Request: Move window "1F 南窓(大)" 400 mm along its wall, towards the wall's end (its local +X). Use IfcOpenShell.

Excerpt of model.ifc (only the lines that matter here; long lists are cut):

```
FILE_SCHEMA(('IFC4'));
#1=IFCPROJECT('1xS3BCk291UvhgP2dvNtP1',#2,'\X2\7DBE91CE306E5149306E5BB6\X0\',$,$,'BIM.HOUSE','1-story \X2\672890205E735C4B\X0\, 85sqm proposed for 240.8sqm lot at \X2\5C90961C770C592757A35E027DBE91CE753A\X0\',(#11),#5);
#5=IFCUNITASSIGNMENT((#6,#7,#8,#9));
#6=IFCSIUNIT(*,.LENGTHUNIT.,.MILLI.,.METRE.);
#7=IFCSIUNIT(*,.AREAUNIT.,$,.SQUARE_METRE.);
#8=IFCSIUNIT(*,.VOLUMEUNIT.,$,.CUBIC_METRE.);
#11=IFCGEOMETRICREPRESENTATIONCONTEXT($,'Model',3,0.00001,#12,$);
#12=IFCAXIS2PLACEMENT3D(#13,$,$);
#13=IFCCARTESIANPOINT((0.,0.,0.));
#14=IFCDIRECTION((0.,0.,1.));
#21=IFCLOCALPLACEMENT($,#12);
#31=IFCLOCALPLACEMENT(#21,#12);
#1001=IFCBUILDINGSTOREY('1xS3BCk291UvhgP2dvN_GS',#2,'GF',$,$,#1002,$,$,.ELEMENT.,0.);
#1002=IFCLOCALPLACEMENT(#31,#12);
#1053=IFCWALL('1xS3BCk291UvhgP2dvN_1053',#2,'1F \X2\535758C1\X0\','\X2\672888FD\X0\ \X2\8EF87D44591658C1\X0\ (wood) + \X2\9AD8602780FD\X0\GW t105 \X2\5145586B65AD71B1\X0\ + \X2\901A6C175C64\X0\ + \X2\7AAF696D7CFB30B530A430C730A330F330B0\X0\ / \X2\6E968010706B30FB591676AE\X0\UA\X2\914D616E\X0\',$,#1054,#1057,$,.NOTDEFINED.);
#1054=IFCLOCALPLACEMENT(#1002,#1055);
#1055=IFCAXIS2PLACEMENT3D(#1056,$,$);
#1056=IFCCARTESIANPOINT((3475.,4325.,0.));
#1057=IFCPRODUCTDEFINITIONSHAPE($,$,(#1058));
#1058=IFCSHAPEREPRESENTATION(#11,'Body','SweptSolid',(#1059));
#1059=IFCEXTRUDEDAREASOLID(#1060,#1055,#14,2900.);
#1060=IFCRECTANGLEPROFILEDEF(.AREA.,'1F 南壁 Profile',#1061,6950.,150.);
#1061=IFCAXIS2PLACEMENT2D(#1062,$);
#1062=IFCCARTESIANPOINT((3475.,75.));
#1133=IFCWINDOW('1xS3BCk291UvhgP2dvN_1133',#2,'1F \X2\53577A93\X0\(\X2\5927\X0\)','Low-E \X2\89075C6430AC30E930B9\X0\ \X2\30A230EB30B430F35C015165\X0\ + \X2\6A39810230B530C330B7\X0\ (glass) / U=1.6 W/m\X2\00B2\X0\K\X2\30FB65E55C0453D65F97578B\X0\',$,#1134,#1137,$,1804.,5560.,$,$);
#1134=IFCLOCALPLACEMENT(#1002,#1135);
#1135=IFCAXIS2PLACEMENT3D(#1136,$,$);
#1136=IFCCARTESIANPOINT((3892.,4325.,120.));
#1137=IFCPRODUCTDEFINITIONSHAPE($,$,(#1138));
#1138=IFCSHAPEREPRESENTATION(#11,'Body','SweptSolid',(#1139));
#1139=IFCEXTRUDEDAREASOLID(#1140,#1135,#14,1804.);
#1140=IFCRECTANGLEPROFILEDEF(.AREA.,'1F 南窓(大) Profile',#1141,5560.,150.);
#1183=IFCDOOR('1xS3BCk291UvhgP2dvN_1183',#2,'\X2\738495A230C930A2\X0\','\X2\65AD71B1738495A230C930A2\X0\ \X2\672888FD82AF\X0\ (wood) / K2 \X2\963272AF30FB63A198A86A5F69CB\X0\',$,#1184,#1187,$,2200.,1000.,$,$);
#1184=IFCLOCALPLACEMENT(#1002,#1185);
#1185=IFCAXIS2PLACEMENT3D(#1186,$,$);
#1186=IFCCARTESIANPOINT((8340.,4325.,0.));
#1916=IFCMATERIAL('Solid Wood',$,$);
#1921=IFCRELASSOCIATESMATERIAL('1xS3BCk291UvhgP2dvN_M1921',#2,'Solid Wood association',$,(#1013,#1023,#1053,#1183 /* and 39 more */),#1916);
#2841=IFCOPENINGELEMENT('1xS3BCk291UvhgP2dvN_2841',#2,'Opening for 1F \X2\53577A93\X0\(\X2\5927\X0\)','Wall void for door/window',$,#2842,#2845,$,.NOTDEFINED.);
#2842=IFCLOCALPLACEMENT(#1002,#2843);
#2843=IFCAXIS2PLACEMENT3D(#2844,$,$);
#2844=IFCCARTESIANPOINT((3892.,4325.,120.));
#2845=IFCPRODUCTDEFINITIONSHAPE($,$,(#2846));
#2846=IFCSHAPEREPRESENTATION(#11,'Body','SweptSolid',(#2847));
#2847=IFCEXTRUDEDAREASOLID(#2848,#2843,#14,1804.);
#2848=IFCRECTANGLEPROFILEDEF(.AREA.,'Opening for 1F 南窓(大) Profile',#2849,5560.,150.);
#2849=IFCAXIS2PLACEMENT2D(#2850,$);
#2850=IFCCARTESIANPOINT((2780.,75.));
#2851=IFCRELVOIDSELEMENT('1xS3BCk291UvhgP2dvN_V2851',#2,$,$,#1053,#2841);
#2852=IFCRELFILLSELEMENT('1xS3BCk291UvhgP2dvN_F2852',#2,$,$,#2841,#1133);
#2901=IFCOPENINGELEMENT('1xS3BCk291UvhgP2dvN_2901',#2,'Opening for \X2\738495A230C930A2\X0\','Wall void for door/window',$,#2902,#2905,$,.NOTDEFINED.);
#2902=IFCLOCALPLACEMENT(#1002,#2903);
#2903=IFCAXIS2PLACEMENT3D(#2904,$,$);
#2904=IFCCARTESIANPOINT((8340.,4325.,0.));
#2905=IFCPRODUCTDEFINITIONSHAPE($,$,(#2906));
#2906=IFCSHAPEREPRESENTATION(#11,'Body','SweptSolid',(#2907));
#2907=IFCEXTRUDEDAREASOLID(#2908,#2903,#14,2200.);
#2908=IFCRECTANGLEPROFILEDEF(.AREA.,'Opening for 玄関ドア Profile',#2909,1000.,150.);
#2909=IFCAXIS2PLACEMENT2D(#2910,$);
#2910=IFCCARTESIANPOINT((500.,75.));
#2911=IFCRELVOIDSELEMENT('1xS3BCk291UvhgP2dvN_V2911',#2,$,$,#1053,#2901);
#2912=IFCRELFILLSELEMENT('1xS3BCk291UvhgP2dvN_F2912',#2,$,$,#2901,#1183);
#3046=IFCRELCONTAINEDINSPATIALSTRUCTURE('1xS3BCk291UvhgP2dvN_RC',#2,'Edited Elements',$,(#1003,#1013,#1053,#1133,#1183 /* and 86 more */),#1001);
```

```python
import ifcopenshell
import ifcopenshell.api.geometry
import ifcopenshell.util.placement

model = ifcopenshell.open("model.ifc")

window = model.by_guid("1xS3BCk291UvhgP2dvN_1133")
opening = window.FillsVoids[0].RelatingOpeningElement
wall = opening.VoidsElements[0].RelatingBuildingElement

wall_matrix = ifcopenshell.util.placement.get_local_placement(wall.ObjectPlacement)
shift = wall_matrix[:3, 0] * 400.0
before = ifcopenshell.util.placement.get_local_placement(window.ObjectPlacement)[:3, 3].copy()

# The window is not placed relative to its opening, so move both.
for product in (opening, window):
    matrix = ifcopenshell.util.placement.get_local_placement(product.ObjectPlacement)
    matrix[:3, 3] += shift
    ifcopenshell.api.geometry.edit_object_placement(model, product=product, matrix=matrix, is_si=False)

after = ifcopenshell.util.placement.get_local_placement(window.ObjectPlacement)[:3, 3]
print("window moved by", (after - before).round(3) + 0.0)

model.write("model_edited.ifc")
```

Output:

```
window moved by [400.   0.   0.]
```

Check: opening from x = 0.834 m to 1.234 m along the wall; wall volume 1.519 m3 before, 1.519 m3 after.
